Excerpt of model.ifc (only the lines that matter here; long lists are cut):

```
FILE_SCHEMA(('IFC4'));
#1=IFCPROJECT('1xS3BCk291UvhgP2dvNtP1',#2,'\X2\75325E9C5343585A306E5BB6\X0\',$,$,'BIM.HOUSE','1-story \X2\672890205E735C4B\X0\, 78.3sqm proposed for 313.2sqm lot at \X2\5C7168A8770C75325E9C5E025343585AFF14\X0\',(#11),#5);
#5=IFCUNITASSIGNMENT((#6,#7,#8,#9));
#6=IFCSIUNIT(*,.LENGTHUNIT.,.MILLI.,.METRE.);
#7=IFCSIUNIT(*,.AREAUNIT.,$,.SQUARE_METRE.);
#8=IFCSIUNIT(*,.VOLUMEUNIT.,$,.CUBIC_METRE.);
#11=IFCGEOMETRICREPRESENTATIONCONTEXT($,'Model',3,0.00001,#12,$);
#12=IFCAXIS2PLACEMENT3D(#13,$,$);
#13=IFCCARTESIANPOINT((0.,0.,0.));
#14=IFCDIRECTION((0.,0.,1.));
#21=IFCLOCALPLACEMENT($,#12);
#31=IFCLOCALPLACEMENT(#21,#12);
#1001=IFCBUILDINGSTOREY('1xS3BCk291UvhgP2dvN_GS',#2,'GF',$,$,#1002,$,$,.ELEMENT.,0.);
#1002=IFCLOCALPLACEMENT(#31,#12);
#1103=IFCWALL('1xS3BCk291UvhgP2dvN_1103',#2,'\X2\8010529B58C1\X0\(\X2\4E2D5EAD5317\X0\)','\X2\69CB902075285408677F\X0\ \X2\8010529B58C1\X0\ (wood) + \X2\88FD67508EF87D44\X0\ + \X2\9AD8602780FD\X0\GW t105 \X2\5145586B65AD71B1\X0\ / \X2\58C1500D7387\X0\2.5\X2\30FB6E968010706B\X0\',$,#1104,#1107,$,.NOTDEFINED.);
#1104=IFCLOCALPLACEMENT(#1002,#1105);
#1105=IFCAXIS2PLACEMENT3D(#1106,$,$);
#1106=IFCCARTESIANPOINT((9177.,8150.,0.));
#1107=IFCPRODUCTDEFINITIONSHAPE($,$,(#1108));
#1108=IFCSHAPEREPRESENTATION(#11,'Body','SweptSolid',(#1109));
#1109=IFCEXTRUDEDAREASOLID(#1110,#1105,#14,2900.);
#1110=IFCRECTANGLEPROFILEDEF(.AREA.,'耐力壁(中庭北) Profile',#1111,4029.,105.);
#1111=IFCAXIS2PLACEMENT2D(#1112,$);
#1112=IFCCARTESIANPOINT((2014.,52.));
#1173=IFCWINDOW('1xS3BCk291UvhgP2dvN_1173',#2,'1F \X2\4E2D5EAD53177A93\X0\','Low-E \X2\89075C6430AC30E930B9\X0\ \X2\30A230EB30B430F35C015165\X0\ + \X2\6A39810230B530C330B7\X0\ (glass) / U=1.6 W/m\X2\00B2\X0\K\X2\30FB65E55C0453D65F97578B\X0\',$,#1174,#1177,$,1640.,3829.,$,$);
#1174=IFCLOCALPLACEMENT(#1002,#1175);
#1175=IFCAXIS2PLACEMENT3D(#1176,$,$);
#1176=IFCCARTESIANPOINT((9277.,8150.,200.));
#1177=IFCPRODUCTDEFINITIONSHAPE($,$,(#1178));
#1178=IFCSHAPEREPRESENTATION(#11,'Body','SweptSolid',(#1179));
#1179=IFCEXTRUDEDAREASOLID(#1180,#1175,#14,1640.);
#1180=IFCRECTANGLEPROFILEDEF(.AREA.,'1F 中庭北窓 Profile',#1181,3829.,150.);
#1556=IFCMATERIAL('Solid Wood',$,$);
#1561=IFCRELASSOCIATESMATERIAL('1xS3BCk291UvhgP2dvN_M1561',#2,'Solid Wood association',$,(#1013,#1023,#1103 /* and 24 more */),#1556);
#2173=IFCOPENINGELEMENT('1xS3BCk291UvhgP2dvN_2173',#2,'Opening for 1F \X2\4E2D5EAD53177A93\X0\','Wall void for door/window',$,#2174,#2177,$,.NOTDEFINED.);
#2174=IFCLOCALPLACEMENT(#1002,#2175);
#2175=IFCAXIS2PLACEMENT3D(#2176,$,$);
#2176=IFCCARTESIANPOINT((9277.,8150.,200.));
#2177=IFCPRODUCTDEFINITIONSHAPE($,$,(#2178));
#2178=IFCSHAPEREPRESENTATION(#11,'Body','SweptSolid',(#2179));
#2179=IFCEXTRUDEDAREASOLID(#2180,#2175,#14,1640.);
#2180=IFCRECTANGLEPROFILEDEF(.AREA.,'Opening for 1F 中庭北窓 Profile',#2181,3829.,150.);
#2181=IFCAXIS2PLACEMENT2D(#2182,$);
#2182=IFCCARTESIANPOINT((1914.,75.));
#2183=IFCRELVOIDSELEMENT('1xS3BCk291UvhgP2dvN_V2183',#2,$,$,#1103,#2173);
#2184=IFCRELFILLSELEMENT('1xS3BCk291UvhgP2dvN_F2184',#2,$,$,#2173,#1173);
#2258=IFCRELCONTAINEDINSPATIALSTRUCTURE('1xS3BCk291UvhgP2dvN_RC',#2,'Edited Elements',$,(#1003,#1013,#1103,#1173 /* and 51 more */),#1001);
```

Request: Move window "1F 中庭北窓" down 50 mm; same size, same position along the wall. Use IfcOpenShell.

```python
import numpy as np
import ifcopenshell
import ifcopenshell.api.geometry
import ifcopenshell.util.placement
import ifcopenshell.util.unit

model = ifcopenshell.open("model.ifc")
unit_scale = ifcopenshell.util.unit.calculate_unit_scale(model)

window = model.by_guid("1xS3BCk291UvhgP2dvN_1173")
opening = window.FillsVoids[0].RelatingOpeningElement
dz = -50.0

shift = np.array([0.0, 0.0, dz])
# The window is not placed relative to its opening, so move both.
for product in (opening, window):
    matrix = ifcopenshell.util.placement.get_local_placement(product.ObjectPlacement)
    matrix[:3, 3] += shift
    ifcopenshell.api.geometry.edit_object_placement(model, product=product, matrix=matrix, is_si=False)

print(f"moved by {dz * unit_scale:+.3f} m")

model.write("model_edited.ifc")
```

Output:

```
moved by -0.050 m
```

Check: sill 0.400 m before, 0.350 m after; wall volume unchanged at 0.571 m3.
